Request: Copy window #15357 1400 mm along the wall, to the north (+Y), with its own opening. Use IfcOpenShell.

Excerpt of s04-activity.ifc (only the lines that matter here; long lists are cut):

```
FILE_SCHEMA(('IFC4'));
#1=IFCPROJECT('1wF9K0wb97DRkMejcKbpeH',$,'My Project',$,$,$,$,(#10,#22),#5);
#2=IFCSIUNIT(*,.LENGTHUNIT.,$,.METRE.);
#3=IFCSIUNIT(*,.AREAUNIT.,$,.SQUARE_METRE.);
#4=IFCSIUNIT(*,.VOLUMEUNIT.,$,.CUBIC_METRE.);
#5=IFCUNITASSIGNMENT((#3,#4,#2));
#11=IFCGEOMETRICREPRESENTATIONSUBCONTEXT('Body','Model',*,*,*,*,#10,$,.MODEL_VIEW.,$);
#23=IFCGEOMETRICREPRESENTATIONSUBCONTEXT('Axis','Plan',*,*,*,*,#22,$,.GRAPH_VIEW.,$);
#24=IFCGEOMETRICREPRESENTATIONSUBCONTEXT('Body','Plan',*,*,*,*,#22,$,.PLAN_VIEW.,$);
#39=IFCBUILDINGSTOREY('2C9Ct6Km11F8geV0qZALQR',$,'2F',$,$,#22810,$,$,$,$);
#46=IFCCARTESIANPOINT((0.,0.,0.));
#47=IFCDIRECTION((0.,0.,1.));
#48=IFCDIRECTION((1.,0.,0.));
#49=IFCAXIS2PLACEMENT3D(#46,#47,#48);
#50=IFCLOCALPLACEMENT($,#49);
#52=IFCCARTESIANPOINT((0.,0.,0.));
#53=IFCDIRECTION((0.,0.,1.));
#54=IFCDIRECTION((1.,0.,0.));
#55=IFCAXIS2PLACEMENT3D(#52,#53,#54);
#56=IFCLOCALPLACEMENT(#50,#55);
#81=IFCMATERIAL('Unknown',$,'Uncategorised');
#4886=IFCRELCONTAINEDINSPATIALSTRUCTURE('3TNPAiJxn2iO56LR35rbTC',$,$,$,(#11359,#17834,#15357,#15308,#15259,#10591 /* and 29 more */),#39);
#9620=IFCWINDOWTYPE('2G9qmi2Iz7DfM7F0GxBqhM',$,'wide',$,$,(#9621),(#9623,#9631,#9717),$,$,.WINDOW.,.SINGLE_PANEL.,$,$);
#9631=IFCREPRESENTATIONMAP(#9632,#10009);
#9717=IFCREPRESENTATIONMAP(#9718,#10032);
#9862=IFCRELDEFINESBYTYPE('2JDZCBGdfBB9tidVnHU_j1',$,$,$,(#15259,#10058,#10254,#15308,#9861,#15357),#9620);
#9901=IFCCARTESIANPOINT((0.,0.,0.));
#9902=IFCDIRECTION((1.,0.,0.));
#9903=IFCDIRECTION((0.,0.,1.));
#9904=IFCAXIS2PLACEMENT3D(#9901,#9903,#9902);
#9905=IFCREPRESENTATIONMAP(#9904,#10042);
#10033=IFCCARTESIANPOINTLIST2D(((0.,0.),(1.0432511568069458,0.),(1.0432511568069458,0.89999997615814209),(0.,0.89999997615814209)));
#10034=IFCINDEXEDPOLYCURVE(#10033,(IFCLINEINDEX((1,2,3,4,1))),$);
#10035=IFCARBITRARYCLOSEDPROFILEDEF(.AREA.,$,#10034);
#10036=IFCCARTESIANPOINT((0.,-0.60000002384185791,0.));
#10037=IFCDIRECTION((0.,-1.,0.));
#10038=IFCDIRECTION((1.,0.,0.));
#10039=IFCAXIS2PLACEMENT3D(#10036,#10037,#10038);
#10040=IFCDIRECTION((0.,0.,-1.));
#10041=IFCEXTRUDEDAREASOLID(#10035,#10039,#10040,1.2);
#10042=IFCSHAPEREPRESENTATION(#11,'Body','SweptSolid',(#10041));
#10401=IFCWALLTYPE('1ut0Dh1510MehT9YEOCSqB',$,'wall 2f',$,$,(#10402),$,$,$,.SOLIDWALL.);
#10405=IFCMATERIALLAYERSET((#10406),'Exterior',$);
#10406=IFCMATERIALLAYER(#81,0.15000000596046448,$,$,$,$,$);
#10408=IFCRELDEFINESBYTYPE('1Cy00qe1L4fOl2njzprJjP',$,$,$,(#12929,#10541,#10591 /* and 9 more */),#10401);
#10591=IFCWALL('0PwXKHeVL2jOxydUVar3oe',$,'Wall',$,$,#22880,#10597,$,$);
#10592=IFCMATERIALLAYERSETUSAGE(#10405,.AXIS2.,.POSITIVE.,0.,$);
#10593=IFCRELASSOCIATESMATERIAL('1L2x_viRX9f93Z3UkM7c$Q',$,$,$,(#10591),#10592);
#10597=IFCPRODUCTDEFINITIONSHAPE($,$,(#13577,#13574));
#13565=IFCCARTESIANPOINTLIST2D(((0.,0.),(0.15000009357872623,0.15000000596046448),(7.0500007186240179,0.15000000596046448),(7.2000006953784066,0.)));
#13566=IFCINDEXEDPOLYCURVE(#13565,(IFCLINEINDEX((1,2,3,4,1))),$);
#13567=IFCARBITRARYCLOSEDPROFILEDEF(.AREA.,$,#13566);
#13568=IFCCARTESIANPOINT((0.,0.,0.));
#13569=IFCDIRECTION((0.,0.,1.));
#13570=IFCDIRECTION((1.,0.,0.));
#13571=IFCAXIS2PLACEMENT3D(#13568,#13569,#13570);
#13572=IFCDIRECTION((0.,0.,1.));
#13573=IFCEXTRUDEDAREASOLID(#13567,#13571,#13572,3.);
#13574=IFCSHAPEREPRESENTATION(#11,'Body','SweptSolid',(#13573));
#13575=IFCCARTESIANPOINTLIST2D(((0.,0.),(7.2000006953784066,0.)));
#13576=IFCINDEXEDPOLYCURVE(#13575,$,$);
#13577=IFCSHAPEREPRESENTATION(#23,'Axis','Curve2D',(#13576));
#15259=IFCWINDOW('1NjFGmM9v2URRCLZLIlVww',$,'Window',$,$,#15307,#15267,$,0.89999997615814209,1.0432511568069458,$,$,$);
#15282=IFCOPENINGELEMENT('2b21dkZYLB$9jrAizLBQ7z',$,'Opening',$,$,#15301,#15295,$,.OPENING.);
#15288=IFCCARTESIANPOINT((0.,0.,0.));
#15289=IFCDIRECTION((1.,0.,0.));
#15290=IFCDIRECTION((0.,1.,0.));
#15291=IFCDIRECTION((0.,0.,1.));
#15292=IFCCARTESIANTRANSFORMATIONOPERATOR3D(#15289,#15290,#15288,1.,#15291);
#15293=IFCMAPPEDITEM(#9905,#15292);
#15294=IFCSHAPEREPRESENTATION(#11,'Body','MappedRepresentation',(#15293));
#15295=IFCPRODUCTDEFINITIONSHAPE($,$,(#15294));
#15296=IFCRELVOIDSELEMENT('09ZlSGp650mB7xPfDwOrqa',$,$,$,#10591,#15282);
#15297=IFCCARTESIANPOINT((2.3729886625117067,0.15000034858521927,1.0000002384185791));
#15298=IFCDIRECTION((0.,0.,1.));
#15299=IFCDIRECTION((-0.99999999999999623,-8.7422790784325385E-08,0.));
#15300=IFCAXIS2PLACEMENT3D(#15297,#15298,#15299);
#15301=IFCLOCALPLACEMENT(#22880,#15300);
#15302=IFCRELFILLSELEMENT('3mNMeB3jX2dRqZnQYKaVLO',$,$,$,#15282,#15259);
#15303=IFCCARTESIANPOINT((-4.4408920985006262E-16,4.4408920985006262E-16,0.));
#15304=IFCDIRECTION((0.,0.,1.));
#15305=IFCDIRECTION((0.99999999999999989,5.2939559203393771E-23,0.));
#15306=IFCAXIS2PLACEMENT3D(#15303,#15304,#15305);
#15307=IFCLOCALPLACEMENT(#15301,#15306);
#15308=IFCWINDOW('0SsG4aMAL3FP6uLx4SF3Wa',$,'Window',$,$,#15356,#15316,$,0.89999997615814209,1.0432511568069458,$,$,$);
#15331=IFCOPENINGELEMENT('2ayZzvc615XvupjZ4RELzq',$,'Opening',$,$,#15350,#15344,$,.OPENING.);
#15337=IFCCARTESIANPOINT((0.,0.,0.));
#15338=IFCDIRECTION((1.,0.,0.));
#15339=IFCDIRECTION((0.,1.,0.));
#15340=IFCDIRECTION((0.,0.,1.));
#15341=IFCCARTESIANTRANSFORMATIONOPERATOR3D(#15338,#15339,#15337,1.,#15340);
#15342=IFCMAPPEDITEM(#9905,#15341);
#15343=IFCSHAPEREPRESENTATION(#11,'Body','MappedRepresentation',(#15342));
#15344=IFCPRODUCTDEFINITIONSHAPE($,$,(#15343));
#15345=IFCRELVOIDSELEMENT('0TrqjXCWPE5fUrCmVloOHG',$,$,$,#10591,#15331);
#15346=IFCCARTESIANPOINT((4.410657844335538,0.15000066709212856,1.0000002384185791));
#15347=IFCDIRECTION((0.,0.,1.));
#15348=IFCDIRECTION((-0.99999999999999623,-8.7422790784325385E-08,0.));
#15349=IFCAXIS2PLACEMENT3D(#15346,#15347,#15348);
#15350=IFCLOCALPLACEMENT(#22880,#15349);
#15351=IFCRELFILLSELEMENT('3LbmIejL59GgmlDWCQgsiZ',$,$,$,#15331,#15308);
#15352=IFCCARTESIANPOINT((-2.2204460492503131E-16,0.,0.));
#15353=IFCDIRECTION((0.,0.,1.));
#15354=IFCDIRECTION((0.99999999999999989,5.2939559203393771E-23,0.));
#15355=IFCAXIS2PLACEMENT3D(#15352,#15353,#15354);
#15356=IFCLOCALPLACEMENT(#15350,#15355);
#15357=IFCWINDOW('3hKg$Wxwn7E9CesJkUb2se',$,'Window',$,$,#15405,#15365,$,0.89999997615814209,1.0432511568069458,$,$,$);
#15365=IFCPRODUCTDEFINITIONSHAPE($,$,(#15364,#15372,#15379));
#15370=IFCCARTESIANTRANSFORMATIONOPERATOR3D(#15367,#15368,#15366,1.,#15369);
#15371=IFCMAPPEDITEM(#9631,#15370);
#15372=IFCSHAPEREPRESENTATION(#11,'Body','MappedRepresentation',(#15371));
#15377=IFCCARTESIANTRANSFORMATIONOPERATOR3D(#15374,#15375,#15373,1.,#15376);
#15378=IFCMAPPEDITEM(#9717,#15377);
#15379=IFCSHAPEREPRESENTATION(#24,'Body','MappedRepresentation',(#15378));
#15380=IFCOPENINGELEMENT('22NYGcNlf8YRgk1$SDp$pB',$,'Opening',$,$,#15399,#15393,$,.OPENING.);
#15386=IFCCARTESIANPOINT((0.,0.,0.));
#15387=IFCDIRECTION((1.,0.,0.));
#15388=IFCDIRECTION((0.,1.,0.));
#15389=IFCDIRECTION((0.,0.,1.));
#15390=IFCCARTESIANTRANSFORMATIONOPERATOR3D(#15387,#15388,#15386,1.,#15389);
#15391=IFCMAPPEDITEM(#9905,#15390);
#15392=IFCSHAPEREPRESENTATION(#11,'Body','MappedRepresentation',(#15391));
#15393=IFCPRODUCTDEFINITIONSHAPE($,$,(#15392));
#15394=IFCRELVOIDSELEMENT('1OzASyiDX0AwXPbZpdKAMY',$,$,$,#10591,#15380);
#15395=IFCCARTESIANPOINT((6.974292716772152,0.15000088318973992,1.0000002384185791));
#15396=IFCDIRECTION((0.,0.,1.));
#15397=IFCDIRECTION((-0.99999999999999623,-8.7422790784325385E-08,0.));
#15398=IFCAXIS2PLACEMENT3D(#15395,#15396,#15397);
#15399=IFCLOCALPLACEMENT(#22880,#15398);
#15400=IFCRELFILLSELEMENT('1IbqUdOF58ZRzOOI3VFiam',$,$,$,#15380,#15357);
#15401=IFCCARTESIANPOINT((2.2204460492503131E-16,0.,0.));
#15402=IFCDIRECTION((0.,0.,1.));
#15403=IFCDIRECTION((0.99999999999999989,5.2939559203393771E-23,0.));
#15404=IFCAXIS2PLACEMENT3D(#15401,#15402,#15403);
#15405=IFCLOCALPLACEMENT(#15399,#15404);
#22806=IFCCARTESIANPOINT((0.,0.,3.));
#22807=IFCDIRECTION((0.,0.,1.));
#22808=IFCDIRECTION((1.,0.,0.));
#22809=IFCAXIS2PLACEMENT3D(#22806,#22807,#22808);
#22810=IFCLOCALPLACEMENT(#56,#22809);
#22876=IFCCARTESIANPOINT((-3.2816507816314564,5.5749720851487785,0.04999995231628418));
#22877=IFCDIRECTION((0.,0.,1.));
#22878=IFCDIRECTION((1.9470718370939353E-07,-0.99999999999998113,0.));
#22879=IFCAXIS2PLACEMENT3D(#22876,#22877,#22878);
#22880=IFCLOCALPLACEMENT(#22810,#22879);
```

```python
import ifcopenshell
import ifcopenshell.api.feature
import ifcopenshell.api.geometry
import ifcopenshell.api.root
import ifcopenshell.geom
import ifcopenshell.util.element
import ifcopenshell.util.placement
import ifcopenshell.util.shape

model = ifcopenshell.open("s04-activity.ifc")
settings = ifcopenshell.geom.settings()


def volume(element):
    """Net volume in cubic metres, openings subtracted."""
    shape = ifcopenshell.geom.create_shape(settings, element)
    return ifcopenshell.util.shape.get_volume(shape.geometry)


window = model.by_guid("3hKg$Wxwn7E9CesJkUb2se")
opening = window.FillsVoids[0].RelatingOpeningElement
wall = opening.VoidsElements[0].RelatingBuildingElement
before = volume(wall)
shift = ifcopenshell.util.placement.get_local_placement(wall.ObjectPlacement)[:3, 0] * -1.4

# copy_class copies the void relationship, type, container and properties, but no geometry.
new_opening = ifcopenshell.api.root.copy_class(model, product=opening)
new_opening.Representation = ifcopenshell.util.element.copy_deep(
    model, opening.Representation, exclude=["IfcGeometricRepresentationContext", "IfcRepresentationMap"]
)
new_window = ifcopenshell.api.root.copy_class(model, product=window)
new_window.Representation = ifcopenshell.util.element.copy_deep(
    model, window.Representation, exclude=["IfcGeometricRepresentationContext", "IfcRepresentationMap"]
)
ifcopenshell.api.feature.add_filling(model, opening=new_opening, element=new_window)

for old, new in ((opening, new_opening), (window, new_window)):
    matrix = ifcopenshell.util.placement.get_local_placement(old.ObjectPlacement)
    matrix[:3, 3] += shift
    ifcopenshell.api.geometry.edit_object_placement(model, product=new, matrix=matrix, is_si=False)

after = volume(wall)

print(f"wall volume {before:.3f} -> {after:.3f} m3")

model.write("s04-activity_v2.ifc")
```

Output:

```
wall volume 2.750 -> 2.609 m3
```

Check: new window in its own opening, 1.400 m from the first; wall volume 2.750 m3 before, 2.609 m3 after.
